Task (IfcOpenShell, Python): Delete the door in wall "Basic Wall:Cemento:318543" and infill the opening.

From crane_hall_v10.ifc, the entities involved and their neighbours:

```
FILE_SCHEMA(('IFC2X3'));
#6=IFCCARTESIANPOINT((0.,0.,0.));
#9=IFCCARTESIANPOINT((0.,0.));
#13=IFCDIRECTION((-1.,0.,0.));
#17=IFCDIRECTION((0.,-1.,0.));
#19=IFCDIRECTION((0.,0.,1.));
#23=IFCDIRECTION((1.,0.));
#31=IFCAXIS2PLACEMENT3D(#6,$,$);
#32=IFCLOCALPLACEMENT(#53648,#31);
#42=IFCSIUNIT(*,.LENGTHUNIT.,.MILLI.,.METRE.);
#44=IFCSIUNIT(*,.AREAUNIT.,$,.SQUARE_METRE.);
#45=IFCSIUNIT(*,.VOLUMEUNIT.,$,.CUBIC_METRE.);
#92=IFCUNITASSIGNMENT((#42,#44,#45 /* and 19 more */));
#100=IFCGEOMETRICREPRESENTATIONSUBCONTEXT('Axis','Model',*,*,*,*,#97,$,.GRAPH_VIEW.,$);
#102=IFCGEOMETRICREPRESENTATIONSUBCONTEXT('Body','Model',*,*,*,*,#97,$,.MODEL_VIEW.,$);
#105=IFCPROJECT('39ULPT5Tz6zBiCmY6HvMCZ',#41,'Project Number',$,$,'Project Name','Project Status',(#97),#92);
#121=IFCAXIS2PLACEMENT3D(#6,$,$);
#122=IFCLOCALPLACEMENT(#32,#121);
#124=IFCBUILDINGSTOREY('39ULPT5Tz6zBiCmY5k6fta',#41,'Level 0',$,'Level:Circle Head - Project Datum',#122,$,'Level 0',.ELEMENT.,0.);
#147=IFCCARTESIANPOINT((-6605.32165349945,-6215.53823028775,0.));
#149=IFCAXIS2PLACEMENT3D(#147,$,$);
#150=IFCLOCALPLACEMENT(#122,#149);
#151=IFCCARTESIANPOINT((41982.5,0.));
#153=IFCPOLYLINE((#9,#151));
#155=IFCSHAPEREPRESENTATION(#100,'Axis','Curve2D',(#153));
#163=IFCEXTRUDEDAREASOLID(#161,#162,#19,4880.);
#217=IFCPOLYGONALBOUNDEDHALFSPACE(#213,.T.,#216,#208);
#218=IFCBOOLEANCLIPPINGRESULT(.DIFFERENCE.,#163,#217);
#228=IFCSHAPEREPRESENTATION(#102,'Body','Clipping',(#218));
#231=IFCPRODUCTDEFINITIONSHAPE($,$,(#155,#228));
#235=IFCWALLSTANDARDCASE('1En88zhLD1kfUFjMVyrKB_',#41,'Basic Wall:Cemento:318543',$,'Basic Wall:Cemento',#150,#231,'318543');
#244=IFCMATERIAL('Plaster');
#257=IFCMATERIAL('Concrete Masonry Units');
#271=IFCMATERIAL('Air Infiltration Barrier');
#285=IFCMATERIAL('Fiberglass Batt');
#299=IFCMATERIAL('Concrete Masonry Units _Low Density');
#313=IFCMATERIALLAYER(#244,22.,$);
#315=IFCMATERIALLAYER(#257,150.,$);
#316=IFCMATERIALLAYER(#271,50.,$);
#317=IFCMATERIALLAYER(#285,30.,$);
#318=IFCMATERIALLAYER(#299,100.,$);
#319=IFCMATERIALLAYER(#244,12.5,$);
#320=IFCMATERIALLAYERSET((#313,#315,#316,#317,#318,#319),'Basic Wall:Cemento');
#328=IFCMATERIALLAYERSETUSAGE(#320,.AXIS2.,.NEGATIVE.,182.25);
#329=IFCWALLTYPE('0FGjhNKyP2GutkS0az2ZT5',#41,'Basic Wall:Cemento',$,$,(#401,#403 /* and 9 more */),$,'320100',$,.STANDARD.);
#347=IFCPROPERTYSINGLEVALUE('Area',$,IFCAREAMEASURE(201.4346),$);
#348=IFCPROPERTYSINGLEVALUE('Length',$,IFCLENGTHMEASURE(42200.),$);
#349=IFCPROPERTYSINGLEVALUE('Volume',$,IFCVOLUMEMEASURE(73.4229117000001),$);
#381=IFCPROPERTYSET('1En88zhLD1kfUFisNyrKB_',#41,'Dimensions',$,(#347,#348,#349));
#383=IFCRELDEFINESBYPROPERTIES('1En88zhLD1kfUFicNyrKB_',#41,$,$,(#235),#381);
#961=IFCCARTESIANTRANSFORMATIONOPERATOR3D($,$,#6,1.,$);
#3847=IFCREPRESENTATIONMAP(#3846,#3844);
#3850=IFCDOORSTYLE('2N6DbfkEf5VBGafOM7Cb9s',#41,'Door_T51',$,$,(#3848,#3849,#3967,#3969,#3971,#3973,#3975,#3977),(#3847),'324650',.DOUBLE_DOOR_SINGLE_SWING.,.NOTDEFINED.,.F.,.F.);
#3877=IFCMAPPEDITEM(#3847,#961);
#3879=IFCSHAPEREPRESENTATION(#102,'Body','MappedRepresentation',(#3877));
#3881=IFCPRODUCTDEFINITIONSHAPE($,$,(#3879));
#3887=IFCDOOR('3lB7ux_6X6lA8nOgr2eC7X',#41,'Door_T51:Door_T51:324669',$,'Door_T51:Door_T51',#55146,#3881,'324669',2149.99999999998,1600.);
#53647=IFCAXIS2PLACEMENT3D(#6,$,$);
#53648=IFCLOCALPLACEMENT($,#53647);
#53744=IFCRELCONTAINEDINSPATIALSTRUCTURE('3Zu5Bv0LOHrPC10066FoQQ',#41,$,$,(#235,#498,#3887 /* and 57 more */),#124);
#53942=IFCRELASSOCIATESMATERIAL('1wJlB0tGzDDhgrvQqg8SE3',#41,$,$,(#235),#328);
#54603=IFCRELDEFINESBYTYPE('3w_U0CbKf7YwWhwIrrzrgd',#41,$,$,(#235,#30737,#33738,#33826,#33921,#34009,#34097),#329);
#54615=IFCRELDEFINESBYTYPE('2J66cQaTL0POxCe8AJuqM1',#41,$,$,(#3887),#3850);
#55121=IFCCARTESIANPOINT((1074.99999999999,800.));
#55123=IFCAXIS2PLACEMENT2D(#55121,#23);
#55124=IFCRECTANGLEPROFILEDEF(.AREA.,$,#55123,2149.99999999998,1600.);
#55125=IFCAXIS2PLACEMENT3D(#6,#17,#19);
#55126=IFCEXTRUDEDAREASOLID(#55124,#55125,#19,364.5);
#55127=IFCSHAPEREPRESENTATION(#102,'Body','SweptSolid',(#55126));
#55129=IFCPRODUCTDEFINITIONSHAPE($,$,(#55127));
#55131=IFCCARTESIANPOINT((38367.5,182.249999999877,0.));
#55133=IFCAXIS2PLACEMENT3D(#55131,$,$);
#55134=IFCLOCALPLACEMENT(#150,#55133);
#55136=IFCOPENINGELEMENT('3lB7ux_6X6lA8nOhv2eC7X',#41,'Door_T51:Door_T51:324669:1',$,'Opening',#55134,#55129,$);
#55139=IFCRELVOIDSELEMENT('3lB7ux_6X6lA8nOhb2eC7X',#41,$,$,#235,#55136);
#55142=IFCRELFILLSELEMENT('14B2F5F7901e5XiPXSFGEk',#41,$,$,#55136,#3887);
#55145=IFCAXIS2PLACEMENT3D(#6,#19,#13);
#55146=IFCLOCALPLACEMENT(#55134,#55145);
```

```python
import ifcopenshell
import ifcopenshell.api.feature
import ifcopenshell.api.pset
import ifcopenshell.api.root
import ifcopenshell.geom
import ifcopenshell.util.element
import ifcopenshell.util.shape
import ifcopenshell.util.unit

model = ifcopenshell.open("crane_hall_v10.ifc")
area_scale = ifcopenshell.util.unit.calculate_unit_scale(model, "AREAUNIT")
volume_scale = ifcopenshell.util.unit.calculate_unit_scale(model, "VOLUMEUNIT")
settings = ifcopenshell.geom.settings()


def volume(element):
    """Net volume in cubic metres, openings subtracted."""
    shape = ifcopenshell.geom.create_shape(settings, element)
    return ifcopenshell.util.shape.get_volume(shape.geometry)


door = model.by_guid("3lB7ux_6X6lA8nOgr2eC7X")
opening = door.FillsVoids[0].RelatingOpeningElement
wall = opening.VoidsElements[0].RelatingBuildingElement
before = volume(wall)

ifcopenshell.api.root.remove_product(model, product=door)
ifcopenshell.api.feature.remove_feature(model, feature=opening)

after = volume(wall)
thickness = 0.3645  # wall thickness in metres

# Update the wall's stored quantities.
pset = model.by_id(ifcopenshell.util.element.get_pset(wall, "Dimensions", should_inherit=False)["id"])
ifcopenshell.api.pset.edit_pset(model, pset=pset, properties={
    "Area": model.create_entity("IfcAreaMeasure", after / thickness / area_scale),
    "Volume": model.create_entity("IfcVolumeMeasure", after / volume_scale),
})

print(f"wall volume {before:.3f} -> {after:.3f} m3")

model.write("crane_hall_v10-out.ifc")
```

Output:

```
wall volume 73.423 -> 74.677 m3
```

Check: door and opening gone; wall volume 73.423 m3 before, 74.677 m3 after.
